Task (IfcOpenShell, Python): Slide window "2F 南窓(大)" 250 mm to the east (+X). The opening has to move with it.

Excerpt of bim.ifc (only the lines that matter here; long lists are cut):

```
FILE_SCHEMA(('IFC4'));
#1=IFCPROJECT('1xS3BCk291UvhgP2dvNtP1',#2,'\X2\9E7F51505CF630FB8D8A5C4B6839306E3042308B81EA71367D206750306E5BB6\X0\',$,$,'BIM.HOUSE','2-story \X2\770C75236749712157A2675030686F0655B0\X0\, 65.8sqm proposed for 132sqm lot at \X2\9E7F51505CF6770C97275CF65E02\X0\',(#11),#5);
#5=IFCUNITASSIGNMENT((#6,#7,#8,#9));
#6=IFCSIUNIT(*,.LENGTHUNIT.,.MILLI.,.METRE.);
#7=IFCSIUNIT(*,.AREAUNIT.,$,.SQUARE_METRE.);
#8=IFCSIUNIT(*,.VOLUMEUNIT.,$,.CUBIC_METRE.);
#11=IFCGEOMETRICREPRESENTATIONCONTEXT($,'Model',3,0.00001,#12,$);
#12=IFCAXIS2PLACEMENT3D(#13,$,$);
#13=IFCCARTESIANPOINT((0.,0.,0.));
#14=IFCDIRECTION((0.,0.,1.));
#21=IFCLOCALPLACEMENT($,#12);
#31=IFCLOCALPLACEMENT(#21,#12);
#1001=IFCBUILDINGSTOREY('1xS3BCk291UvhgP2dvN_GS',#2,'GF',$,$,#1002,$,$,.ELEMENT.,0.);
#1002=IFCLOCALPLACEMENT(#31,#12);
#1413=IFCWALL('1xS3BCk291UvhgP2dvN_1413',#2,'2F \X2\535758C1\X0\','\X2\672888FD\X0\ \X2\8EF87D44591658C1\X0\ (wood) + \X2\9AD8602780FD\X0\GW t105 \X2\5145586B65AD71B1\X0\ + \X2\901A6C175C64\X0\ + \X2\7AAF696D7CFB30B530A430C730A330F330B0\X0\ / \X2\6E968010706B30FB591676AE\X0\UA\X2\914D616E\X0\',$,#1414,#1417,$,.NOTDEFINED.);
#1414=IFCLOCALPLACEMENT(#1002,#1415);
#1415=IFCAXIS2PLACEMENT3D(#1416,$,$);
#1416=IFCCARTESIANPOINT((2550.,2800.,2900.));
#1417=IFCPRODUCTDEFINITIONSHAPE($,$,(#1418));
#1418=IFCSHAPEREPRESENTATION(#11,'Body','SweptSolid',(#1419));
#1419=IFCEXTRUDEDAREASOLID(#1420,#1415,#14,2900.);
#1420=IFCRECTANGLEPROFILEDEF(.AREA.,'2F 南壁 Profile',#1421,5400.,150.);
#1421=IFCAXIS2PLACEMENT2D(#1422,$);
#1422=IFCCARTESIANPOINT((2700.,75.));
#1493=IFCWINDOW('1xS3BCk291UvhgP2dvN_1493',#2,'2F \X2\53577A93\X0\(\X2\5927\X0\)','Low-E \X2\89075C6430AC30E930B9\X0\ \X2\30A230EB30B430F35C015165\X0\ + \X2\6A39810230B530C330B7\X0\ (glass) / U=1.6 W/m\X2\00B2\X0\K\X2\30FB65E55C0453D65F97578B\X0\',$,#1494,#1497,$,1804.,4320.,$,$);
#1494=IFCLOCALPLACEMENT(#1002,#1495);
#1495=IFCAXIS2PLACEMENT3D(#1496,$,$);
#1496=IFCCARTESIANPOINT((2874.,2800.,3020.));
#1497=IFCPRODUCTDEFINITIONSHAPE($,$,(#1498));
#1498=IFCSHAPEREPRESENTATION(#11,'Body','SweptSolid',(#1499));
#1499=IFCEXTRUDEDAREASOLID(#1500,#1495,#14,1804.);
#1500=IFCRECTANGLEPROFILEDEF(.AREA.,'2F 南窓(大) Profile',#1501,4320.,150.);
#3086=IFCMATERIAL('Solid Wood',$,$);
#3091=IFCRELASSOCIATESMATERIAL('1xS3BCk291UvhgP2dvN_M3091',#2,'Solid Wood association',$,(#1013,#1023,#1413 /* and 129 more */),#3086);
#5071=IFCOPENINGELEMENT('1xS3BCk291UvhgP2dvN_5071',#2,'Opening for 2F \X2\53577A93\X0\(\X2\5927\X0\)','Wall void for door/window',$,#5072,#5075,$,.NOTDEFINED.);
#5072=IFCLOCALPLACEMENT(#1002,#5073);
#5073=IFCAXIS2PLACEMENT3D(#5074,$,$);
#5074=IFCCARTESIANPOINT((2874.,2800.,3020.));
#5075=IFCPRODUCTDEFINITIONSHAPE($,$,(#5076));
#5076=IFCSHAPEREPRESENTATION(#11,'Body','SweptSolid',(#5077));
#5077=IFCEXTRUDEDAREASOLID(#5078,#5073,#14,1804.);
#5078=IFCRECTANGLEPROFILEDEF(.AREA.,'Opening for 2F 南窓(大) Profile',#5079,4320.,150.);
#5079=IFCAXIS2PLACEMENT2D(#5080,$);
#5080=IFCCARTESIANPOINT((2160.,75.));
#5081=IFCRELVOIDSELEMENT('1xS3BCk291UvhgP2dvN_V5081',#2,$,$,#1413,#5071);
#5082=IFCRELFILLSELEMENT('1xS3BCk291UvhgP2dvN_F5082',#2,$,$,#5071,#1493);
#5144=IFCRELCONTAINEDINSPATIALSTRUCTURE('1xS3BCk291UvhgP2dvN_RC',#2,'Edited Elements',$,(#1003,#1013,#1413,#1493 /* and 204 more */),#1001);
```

```python
import ifcopenshell
import ifcopenshell.api.geometry
import ifcopenshell.util.placement
import ifcopenshell.util.unit

model = ifcopenshell.open("bim.ifc")
unit_scale = ifcopenshell.util.unit.calculate_unit_scale(model)

window = model.by_guid("1xS3BCk291UvhgP2dvN_1493")
opening = window.FillsVoids[0].RelatingOpeningElement
wall = opening.VoidsElements[0].RelatingBuildingElement

wall_matrix = ifcopenshell.util.placement.get_local_placement(wall.ObjectPlacement)
shift = wall_matrix[:3, 0] * 0.25 / unit_scale
before = ifcopenshell.util.placement.get_local_placement(window.ObjectPlacement)[:3, 3].copy()

# The window is not placed relative to its opening, so move both.
for product in (opening, window):
    matrix = ifcopenshell.util.placement.get_local_placement(product.ObjectPlacement)
    matrix[:3, 3] += shift
    ifcopenshell.api.geometry.edit_object_placement(model, product=product, matrix=matrix, is_si=False)

after = ifcopenshell.util.placement.get_local_placement(window.ObjectPlacement)[:3, 3]
print("window moved by", (after - before).round(3) + 0.0)

model.write("bim_rev.ifc")
```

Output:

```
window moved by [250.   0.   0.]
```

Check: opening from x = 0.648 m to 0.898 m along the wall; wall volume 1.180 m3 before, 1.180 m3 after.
